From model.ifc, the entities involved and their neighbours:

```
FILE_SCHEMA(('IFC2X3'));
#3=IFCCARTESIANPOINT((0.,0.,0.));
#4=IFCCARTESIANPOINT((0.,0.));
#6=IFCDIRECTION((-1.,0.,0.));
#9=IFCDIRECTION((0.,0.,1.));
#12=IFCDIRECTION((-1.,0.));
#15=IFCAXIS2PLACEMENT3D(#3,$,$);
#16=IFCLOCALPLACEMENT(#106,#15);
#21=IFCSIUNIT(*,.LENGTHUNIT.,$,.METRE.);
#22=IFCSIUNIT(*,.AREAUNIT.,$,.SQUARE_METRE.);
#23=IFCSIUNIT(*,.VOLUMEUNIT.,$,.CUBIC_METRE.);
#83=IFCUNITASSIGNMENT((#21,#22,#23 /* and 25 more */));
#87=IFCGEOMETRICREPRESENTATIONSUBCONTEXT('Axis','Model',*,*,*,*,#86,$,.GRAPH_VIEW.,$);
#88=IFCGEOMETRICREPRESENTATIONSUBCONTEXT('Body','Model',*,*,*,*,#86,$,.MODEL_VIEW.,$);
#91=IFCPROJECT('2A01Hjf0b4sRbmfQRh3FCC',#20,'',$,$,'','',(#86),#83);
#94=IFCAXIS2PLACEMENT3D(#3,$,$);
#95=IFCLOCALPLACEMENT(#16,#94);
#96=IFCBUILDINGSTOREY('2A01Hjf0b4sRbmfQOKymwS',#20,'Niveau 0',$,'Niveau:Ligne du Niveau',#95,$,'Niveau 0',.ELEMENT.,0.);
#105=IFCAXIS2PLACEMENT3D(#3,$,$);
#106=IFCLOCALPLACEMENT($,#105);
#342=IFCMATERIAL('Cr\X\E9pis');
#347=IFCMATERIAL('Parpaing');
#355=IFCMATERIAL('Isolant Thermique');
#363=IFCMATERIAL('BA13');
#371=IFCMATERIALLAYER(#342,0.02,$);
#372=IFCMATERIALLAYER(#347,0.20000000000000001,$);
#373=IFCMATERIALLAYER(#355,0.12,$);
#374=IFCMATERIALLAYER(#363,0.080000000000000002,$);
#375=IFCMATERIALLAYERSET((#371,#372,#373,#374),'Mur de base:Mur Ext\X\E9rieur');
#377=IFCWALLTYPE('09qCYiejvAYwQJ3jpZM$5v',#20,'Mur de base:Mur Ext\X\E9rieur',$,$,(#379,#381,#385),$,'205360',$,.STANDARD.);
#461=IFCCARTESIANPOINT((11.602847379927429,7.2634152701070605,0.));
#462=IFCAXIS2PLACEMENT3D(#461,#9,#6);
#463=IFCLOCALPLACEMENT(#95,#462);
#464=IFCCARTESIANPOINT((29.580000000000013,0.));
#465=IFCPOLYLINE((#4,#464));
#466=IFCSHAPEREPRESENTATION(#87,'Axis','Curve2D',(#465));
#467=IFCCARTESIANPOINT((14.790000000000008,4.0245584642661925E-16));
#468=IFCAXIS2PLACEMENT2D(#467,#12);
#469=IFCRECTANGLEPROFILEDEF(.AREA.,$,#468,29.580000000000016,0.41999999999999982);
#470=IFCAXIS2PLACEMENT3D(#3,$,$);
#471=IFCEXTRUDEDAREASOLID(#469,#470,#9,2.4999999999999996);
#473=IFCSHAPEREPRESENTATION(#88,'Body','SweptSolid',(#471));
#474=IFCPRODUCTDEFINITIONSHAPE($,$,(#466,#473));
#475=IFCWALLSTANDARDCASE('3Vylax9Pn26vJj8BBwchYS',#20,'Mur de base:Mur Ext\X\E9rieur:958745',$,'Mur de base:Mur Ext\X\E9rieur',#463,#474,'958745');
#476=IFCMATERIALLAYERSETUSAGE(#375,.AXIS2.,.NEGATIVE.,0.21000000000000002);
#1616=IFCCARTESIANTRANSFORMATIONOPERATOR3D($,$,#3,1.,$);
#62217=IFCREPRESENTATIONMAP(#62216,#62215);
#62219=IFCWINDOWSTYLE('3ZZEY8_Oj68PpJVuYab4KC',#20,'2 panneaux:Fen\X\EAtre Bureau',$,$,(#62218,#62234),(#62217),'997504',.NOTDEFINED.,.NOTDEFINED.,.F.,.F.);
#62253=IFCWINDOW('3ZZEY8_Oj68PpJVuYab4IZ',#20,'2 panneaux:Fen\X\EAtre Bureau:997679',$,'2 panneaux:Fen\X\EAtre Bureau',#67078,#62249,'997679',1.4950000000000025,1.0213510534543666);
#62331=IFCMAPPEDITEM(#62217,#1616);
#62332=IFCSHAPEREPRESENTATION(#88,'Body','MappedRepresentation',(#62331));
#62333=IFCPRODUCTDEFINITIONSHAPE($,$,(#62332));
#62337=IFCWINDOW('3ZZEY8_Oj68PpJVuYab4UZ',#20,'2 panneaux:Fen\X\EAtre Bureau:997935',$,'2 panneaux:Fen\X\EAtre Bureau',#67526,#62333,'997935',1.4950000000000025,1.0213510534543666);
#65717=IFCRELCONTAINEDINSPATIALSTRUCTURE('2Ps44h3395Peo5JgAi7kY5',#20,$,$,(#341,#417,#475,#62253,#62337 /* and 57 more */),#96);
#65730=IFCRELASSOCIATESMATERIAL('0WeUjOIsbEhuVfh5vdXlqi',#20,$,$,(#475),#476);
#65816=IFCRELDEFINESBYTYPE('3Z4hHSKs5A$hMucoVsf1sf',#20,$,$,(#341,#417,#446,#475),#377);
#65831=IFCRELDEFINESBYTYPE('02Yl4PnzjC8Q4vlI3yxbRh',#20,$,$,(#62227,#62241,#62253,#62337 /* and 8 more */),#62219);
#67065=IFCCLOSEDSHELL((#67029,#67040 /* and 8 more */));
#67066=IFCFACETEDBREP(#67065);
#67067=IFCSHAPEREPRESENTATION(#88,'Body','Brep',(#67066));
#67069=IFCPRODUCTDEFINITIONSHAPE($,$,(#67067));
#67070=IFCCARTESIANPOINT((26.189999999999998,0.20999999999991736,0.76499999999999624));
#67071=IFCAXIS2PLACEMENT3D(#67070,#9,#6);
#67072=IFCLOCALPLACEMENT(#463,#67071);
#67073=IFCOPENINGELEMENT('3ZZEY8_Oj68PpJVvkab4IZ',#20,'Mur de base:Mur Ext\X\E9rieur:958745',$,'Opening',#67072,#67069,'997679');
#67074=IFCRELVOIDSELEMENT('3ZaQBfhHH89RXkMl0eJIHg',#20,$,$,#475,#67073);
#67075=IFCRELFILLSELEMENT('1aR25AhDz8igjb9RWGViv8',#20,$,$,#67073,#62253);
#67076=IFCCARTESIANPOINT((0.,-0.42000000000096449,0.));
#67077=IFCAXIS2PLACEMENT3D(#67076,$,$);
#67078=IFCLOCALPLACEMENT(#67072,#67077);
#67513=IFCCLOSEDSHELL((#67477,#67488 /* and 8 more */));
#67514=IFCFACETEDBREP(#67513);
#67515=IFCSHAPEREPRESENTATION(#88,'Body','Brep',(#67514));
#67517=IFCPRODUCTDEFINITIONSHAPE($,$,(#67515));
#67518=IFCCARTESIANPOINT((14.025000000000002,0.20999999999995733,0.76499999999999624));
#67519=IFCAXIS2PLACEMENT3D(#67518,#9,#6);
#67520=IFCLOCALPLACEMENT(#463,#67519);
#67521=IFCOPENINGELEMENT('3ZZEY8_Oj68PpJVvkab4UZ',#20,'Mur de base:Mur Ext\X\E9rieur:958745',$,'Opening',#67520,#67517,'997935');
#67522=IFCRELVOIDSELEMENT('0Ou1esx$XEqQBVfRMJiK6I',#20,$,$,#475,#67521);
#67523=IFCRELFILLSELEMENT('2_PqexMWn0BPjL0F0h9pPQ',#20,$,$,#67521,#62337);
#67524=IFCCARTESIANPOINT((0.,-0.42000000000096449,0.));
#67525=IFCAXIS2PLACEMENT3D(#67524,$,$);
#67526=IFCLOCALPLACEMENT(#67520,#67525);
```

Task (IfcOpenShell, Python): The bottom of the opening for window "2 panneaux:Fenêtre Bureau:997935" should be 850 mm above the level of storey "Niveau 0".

```python
import numpy as np
import ifcopenshell
import ifcopenshell.api.geometry
import ifcopenshell.geom
import ifcopenshell.util.element
import ifcopenshell.util.placement
import ifcopenshell.util.shape
import ifcopenshell.util.unit

model = ifcopenshell.open("model.ifc")
unit_scale = ifcopenshell.util.unit.calculate_unit_scale(model)

window = model.by_guid("3ZZEY8_Oj68PpJVuYab4UZ")
opening = window.FillsVoids[0].RelatingOpeningElement
storey = ifcopenshell.util.element.get_container(window, ifc_class="IfcBuildingStorey")
level = ifcopenshell.util.placement.get_local_placement(storey.ObjectPlacement)[2, 3]

# The opening's origin need not be at the sill, so measure its lowest point.
shape = ifcopenshell.geom.create_shape(ifcopenshell.geom.settings(), opening)
bottom = ifcopenshell.util.shape.get_shape_bottom_elevation(shape, shape.geometry) / unit_scale
dz = level + 0.85 - bottom

shift = np.array([0.0, 0.0, dz])
# The window is placed relative to its opening, so it follows when the opening moves.
matrix = ifcopenshell.util.placement.get_local_placement(opening.ObjectPlacement)
matrix[:3, 3] += shift
ifcopenshell.api.geometry.edit_object_placement(
    model, product=opening, matrix=matrix, is_si=False, should_transform_children=True
)

print(f"moved by {dz * unit_scale:+.3f} m")

model.write("model_rev.ifc")
```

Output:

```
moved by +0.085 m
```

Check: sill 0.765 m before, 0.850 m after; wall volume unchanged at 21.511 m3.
